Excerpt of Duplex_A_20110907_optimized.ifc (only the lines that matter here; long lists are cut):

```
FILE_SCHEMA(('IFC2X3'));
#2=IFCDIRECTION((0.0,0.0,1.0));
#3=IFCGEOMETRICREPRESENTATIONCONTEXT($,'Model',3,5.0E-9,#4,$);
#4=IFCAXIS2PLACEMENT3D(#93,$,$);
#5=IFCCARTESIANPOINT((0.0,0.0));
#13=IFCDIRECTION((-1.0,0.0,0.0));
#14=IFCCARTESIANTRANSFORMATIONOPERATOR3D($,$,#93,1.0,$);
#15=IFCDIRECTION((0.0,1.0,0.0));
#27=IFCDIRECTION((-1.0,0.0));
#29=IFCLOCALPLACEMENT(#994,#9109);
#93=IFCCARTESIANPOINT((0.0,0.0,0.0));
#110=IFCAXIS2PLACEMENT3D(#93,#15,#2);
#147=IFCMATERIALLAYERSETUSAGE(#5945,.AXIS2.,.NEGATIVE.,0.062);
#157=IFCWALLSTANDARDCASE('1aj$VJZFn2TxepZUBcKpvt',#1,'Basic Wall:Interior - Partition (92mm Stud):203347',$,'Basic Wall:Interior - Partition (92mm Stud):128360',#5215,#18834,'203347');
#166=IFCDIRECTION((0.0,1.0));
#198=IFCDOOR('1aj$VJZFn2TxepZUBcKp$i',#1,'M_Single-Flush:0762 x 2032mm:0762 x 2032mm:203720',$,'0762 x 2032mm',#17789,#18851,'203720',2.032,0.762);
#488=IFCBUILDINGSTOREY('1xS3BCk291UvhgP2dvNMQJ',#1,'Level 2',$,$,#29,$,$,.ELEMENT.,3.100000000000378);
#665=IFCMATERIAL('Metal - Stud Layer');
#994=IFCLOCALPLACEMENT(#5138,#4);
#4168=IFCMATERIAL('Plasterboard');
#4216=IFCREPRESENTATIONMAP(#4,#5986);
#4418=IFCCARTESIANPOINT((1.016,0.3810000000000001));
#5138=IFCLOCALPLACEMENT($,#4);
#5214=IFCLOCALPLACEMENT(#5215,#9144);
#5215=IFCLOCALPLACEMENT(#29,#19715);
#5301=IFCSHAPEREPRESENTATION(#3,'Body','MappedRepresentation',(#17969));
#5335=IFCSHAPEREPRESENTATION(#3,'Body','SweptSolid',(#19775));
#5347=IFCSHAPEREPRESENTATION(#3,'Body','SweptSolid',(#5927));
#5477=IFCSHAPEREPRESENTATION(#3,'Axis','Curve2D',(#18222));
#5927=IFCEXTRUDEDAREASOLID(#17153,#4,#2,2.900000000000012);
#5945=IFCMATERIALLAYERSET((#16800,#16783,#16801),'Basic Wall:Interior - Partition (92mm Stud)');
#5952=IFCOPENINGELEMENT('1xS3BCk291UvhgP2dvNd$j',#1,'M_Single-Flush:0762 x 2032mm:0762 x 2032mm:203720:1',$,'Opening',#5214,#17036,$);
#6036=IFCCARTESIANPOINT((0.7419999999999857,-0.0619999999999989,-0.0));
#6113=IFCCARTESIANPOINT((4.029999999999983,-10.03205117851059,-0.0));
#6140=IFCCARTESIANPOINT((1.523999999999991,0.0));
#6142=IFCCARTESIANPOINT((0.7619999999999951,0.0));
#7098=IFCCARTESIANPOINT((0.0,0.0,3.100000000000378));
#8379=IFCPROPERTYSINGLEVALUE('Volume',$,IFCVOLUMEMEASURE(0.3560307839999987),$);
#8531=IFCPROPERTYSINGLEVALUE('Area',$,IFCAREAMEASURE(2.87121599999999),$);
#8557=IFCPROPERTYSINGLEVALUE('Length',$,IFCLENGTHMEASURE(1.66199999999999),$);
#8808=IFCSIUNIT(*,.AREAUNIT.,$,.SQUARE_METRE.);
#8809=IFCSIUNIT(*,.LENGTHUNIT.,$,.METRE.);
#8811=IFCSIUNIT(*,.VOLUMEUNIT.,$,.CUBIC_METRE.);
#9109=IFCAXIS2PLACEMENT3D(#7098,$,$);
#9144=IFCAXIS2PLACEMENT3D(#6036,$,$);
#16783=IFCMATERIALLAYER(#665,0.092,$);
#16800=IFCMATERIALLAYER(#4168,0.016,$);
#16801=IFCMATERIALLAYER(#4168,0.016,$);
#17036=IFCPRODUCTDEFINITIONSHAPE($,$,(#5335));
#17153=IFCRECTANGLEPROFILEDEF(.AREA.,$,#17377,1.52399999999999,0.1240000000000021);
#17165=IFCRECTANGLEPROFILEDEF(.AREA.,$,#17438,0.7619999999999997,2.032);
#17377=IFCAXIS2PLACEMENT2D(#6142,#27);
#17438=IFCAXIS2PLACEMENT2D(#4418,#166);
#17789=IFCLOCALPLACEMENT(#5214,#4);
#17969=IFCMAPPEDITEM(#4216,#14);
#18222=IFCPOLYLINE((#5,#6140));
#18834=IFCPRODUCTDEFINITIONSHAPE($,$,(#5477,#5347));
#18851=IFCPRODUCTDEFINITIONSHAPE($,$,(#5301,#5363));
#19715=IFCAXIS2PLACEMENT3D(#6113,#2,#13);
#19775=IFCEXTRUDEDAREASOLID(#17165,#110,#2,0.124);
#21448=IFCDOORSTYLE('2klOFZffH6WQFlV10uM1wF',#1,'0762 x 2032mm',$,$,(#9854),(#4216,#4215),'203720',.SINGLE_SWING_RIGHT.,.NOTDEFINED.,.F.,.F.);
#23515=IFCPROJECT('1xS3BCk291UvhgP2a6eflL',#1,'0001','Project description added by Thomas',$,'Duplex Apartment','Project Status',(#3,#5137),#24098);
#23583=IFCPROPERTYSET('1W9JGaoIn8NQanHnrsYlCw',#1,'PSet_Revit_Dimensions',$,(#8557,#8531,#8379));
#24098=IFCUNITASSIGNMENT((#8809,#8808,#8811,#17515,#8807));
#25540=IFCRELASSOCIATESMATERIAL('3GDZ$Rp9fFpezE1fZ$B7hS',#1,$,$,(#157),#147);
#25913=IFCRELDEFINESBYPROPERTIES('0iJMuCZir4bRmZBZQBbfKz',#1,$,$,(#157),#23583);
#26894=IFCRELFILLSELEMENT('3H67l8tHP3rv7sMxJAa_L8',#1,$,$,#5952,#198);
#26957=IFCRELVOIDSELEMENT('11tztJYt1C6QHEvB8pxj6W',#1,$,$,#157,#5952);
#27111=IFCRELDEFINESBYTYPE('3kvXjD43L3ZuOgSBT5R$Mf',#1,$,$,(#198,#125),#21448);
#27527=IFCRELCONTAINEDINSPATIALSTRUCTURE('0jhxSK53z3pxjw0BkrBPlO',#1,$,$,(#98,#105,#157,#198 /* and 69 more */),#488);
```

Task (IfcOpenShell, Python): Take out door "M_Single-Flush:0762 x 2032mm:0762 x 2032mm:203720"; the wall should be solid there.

```python
import ifcopenshell
import ifcopenshell.api.feature
import ifcopenshell.api.pset
import ifcopenshell.api.root
import ifcopenshell.geom
import ifcopenshell.util.element
import ifcopenshell.util.shape
import ifcopenshell.util.unit

model = ifcopenshell.open("Duplex_A_20110907_optimized.ifc")
area_scale = ifcopenshell.util.unit.calculate_unit_scale(model, "AREAUNIT")
volume_scale = ifcopenshell.util.unit.calculate_unit_scale(model, "VOLUMEUNIT")
settings = ifcopenshell.geom.settings()


def volume(element):
    """Net volume in cubic metres, openings subtracted."""
    shape = ifcopenshell.geom.create_shape(settings, element)
    return ifcopenshell.util.shape.get_volume(shape.geometry)


door = model.by_id(198)
opening = door.FillsVoids[0].RelatingOpeningElement
wall = opening.VoidsElements[0].RelatingBuildingElement
before = volume(wall)

ifcopenshell.api.root.remove_product(model, product=door)
ifcopenshell.api.feature.remove_feature(model, feature=opening)

after = volume(wall)
thickness = 0.124  # wall thickness in metres

# Update the wall's stored quantities.
pset = model.by_id(ifcopenshell.util.element.get_pset(wall, "PSet_Revit_Dimensions", should_inherit=False)["id"])
ifcopenshell.api.pset.edit_pset(model, pset=pset, properties={
    "Area": model.create_entity("IfcAreaMeasure", after / thickness / area_scale),
    "Volume": model.create_entity("IfcVolumeMeasure", after / volume_scale),
})

print(f"wall volume {before:.3f} -> {after:.3f} m3")

model.write("Duplex_A_20110907_optimized-out.ifc")
```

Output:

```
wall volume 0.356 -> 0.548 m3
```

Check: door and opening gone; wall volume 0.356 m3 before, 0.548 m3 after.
